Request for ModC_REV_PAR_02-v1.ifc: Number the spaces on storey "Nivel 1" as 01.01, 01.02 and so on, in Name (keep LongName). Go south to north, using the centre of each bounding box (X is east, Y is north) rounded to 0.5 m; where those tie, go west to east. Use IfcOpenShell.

First a look at what the model holds.

```python
import ifcopenshell
import ifcopenshell.util.element
import ifcopenshell.util.placement

model = ifcopenshell.open("ModC_REV_PAR_02-v1.ifc")
print(model.schema)
storey = next(s for s in model.by_type("IfcBuildingStorey") if s.Name == "Nivel 1")
spaces = [e for e in ifcopenshell.util.element.get_decomposition(storey) if e.is_a("IfcSpace")]
for e in sorted(spaces, key=lambda e: e.id()):
    origin = ifcopenshell.util.placement.get_local_placement(e.ObjectPlacement)[:3, 3]
    print(e.id(), e.Name, e.LongName, origin.round(2) + 0.0, sep=" | ")
```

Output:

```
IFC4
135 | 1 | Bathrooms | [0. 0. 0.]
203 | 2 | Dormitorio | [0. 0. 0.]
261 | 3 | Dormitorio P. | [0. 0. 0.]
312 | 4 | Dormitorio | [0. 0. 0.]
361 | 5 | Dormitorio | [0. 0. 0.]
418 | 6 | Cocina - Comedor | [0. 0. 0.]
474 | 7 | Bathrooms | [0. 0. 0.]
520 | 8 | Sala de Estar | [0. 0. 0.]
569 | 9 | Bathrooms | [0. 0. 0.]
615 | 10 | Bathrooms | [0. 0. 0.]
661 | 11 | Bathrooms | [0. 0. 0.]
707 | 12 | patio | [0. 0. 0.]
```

```python
import ifcopenshell
import ifcopenshell.geom
import ifcopenshell.util.element
import ifcopenshell.util.shape

model = ifcopenshell.open("ModC_REV_PAR_02-v1.ifc")
settings = ifcopenshell.geom.settings()
settings.set("use-world-coords", True)


def centre(element):
    shape = ifcopenshell.geom.create_shape(settings, element)
    return ifcopenshell.util.shape.get_bbox_centroid(shape.geometry)


storey = next(s for s in model.by_type("IfcBuildingStorey") if s.Name == "Nivel 1")
spaces = [e for e in ifcopenshell.util.element.get_decomposition(storey) if e.is_a("IfcSpace")]

# Insertion points can sit at a corner or the storey origin, so sort by the geometry (in metres).
centres = {e: centre(e) for e in spaces}
spaces.sort(key=lambda e: (round(centres[e][1] / 0.5), centres[e][0]))

for i, e in enumerate(spaces, start=1):
    number = f"01.{i:02d}"
    e.Name = number
    print(e.id(), number)

model.write("ModC_REV_PAR_02-v1_v2.ifc")
```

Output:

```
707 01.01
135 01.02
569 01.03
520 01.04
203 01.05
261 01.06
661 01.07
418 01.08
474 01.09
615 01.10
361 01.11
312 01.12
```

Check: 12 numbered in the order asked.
